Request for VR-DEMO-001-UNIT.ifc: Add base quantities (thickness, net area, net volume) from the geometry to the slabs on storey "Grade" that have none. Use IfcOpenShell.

First a look at what the model holds.

```python
import ifcopenshell
import ifcopenshell.util.element
import ifcopenshell.util.unit

model = ifcopenshell.open("VR-DEMO-001-UNIT.ifc")
print(model.schema)
for unit_type in ("LENGTHUNIT", "AREAUNIT", "VOLUMEUNIT"):
    print(unit_type, ifcopenshell.util.unit.calculate_unit_scale(model, unit_type))
storey = next(s for s in model.by_type("IfcBuildingStorey") if s.Name == "Grade")
slabs = [e for e in ifcopenshell.util.element.get_decomposition(storey) if e.is_a("IfcSlab")]
for e in sorted(slabs, key=lambda e: e.id()):
    print(e.id(), e.is_a(), e.Name, list(ifcopenshell.util.element.get_psets(e, qtos_only=True)), sep=" | ")
```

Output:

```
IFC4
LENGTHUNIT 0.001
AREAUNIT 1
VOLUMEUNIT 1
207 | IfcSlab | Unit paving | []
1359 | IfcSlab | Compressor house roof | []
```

```python
import ifcopenshell
import ifcopenshell.api.pset
import ifcopenshell.geom
import ifcopenshell.util.element
import ifcopenshell.util.shape
import ifcopenshell.util.unit

model = ifcopenshell.open("VR-DEMO-001-UNIT.ifc")
unit_scale = ifcopenshell.util.unit.calculate_unit_scale(model)
area_scale = ifcopenshell.util.unit.calculate_unit_scale(model, "AREAUNIT")
volume_scale = ifcopenshell.util.unit.calculate_unit_scale(model, "VOLUMEUNIT")
settings = ifcopenshell.geom.settings()

storey = next(s for s in model.by_type("IfcBuildingStorey") if s.Name == "Grade")
slabs = [e for e in ifcopenshell.util.element.get_decomposition(storey) if e.is_a("IfcSlab")]

for e in sorted(slabs, key=lambda e: e.id()):
    if ifcopenshell.util.element.get_psets(e, qtos_only=True, should_inherit=False):
        continue
    # Geometry comes back in metres, in the element's own axes.
    shape = ifcopenshell.geom.create_shape(settings, e)
    values = {
        "Width": ifcopenshell.util.shape.get_z(shape.geometry) / unit_scale,
        "NetArea": ifcopenshell.util.shape.get_footprint_area(shape.geometry) / area_scale,
        "NetVolume": ifcopenshell.util.shape.get_volume(shape.geometry) / volume_scale,
    }
    qto = ifcopenshell.api.pset.add_qto(model, product=e, name="Qto_SlabBaseQuantities")
    ifcopenshell.api.pset.edit_qto(model, qto=qto, properties=values)
    print(e.id(), {k: round(v, 3) for k, v in values.items()})

model.write("VR-DEMO-001-UNIT_edited.ifc")
```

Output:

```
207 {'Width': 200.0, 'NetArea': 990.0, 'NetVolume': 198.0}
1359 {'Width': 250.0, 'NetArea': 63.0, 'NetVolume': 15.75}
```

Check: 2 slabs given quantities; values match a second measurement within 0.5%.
